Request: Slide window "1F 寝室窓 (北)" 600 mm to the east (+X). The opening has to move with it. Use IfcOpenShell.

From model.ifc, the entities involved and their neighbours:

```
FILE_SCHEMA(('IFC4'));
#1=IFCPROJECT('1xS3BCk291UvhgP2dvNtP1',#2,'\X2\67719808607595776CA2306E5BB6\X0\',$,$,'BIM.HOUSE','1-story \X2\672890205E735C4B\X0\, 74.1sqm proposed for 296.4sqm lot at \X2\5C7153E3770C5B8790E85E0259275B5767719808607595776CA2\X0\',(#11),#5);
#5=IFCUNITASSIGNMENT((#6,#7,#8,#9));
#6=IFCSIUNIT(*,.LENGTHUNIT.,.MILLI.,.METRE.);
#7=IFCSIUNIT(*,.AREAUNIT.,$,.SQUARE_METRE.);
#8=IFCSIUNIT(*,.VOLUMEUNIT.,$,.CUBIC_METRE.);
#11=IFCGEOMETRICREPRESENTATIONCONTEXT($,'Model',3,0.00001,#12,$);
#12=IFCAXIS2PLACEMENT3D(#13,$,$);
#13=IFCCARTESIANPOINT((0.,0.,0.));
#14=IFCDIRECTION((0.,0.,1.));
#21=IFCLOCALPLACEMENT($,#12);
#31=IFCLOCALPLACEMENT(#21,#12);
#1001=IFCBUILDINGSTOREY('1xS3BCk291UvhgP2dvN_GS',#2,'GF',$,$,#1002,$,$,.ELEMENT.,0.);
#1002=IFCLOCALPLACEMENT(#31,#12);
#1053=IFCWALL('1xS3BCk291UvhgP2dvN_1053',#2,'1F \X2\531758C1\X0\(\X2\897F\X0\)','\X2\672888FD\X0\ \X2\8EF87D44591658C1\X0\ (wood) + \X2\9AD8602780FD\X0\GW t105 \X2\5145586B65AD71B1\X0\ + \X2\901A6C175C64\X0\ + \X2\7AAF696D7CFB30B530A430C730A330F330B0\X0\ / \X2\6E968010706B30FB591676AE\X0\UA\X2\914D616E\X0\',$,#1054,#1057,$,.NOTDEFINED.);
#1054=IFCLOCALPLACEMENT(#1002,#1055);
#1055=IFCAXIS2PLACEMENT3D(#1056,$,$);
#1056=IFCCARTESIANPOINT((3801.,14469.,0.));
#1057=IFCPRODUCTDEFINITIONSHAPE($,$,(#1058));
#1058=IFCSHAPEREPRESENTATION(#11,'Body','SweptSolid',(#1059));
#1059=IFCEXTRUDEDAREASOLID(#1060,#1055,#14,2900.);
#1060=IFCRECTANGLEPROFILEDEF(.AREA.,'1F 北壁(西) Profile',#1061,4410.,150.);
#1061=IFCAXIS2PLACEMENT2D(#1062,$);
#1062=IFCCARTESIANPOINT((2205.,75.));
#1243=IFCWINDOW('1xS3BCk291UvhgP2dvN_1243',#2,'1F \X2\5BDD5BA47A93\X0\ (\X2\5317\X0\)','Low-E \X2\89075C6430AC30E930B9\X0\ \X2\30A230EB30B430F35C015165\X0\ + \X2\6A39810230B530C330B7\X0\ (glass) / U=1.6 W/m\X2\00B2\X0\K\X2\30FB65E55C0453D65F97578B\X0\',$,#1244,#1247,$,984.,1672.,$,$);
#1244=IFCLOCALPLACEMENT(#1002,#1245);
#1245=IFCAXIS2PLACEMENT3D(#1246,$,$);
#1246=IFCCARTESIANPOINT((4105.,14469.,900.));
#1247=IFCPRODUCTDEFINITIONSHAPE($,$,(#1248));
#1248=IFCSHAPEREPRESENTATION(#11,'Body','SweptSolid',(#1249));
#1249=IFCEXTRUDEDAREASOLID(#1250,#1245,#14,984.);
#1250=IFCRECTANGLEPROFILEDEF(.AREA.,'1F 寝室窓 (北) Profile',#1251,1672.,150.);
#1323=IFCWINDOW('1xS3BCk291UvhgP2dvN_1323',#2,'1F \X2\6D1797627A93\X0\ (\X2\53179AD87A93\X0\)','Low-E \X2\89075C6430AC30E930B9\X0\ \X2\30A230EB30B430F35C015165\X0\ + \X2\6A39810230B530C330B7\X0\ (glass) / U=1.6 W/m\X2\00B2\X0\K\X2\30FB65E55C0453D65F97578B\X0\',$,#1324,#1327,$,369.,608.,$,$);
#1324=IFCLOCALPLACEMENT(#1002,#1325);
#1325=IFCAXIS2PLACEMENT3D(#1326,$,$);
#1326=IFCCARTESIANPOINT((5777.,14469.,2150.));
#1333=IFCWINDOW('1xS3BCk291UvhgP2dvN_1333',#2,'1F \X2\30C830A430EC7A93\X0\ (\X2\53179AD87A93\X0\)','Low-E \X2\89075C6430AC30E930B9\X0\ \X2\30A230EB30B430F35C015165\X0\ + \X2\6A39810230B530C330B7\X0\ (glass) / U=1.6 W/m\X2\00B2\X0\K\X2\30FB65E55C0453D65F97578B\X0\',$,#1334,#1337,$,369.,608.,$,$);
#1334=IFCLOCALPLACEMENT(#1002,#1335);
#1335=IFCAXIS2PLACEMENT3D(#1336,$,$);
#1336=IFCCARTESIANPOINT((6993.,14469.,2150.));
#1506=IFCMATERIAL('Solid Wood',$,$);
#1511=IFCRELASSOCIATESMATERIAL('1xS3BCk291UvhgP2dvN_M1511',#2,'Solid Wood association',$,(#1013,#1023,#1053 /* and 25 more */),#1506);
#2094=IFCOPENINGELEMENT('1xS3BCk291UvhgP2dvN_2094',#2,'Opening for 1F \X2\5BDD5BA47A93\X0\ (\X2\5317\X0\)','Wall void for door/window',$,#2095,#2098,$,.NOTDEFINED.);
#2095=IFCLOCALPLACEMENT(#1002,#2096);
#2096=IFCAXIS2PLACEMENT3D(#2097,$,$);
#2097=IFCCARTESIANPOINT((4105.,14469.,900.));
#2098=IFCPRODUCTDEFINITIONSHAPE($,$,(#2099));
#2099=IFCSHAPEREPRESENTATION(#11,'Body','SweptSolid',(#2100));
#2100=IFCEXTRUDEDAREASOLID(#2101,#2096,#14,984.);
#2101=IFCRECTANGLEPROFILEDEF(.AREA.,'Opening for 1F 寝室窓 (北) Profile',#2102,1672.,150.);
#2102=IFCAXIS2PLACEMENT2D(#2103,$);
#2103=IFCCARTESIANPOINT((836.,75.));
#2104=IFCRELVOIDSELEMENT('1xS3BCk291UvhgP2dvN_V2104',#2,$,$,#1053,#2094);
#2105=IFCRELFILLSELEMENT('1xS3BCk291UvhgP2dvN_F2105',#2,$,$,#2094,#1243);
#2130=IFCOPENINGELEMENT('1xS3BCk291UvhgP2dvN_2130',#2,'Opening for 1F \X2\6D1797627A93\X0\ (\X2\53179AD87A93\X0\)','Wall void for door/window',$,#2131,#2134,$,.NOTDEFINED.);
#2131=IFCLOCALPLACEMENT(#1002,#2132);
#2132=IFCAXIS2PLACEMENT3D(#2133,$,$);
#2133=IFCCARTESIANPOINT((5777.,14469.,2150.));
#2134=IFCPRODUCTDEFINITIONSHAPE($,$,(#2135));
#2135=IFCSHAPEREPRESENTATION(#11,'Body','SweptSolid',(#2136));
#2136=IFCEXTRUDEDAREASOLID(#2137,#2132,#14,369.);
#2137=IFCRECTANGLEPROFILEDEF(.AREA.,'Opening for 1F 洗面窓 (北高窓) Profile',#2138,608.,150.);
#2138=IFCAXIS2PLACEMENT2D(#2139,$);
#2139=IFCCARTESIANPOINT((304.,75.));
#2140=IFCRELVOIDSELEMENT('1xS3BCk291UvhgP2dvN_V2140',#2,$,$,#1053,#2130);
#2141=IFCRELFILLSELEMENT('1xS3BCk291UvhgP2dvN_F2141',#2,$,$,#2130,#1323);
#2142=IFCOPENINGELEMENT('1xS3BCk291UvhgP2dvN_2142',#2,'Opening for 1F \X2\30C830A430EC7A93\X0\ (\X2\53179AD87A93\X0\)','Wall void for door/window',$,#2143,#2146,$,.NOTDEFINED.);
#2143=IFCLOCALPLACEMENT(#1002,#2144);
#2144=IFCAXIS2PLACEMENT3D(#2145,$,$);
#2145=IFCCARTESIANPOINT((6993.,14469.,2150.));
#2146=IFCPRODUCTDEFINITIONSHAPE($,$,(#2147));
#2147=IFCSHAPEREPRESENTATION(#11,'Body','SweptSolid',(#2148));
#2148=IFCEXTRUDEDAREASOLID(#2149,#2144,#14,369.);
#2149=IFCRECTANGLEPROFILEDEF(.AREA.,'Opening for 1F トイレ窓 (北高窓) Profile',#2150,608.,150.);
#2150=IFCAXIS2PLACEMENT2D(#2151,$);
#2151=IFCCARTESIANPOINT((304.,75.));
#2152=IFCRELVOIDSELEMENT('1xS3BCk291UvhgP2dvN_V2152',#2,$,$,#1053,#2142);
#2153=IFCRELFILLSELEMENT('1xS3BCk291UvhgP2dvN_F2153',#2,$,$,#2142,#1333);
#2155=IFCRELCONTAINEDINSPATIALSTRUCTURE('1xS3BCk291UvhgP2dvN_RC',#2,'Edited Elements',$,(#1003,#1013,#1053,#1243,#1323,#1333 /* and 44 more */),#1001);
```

```python
import ifcopenshell
import ifcopenshell.api.geometry
import ifcopenshell.util.placement
import ifcopenshell.util.unit

model = ifcopenshell.open("model.ifc")
unit_scale = ifcopenshell.util.unit.calculate_unit_scale(model)

window = model.by_guid("1xS3BCk291UvhgP2dvN_1243")
opening = window.FillsVoids[0].RelatingOpeningElement
wall = opening.VoidsElements[0].RelatingBuildingElement

wall_matrix = ifcopenshell.util.placement.get_local_placement(wall.ObjectPlacement)
shift = wall_matrix[:3, 0] * 0.6 / unit_scale
before = ifcopenshell.util.placement.get_local_placement(window.ObjectPlacement)[:3, 3].copy()

# The window is not placed relative to its opening, so move both.
for product in (opening, window):
    matrix = ifcopenshell.util.placement.get_local_placement(product.ObjectPlacement)
    matrix[:3, 3] += shift
    ifcopenshell.api.geometry.edit_object_placement(model, product=product, matrix=matrix, is_si=False)

after = ifcopenshell.util.placement.get_local_placement(window.ObjectPlacement)[:3, 3]
print("window moved by", (after - before).round(3) + 0.0)

model.write("model-out.ifc")
```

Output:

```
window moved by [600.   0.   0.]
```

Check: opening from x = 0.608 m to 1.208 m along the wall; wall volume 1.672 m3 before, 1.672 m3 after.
